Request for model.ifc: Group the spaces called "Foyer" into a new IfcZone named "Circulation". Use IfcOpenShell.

First a look at what the model holds.

```python
import ifcopenshell

model = ifcopenshell.open("model.ifc")
print(model.schema)
seen = {}
for space in model.by_type("IfcSpace"):
    seen[space.LongName] = seen.get(space.LongName, 0) + 1
for name, count in sorted(seen.items(), key=str):
    print(count, "x", name)
print("zones:", [z.Name for z in model.by_type("IfcZone")][:20])
```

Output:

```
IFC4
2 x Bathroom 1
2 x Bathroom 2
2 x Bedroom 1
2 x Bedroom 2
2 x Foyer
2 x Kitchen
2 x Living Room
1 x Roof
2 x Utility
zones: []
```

```python
import ifcopenshell
import ifcopenshell.api.group
import ifcopenshell.api.root

model = ifcopenshell.open("model.ifc")

names = {"Foyer"}
spaces = [s for s in model.by_type("IfcSpace") if s.LongName in names]

zone = ifcopenshell.api.root.create_entity(model, ifc_class="IfcZone", name="Circulation")
ifcopenshell.api.group.assign_group(model, products=spaces, group=zone)
print(len(spaces), "spaces in", zone.Name)

model.write("model_updated.ifc")
```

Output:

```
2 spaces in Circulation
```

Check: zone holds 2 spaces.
